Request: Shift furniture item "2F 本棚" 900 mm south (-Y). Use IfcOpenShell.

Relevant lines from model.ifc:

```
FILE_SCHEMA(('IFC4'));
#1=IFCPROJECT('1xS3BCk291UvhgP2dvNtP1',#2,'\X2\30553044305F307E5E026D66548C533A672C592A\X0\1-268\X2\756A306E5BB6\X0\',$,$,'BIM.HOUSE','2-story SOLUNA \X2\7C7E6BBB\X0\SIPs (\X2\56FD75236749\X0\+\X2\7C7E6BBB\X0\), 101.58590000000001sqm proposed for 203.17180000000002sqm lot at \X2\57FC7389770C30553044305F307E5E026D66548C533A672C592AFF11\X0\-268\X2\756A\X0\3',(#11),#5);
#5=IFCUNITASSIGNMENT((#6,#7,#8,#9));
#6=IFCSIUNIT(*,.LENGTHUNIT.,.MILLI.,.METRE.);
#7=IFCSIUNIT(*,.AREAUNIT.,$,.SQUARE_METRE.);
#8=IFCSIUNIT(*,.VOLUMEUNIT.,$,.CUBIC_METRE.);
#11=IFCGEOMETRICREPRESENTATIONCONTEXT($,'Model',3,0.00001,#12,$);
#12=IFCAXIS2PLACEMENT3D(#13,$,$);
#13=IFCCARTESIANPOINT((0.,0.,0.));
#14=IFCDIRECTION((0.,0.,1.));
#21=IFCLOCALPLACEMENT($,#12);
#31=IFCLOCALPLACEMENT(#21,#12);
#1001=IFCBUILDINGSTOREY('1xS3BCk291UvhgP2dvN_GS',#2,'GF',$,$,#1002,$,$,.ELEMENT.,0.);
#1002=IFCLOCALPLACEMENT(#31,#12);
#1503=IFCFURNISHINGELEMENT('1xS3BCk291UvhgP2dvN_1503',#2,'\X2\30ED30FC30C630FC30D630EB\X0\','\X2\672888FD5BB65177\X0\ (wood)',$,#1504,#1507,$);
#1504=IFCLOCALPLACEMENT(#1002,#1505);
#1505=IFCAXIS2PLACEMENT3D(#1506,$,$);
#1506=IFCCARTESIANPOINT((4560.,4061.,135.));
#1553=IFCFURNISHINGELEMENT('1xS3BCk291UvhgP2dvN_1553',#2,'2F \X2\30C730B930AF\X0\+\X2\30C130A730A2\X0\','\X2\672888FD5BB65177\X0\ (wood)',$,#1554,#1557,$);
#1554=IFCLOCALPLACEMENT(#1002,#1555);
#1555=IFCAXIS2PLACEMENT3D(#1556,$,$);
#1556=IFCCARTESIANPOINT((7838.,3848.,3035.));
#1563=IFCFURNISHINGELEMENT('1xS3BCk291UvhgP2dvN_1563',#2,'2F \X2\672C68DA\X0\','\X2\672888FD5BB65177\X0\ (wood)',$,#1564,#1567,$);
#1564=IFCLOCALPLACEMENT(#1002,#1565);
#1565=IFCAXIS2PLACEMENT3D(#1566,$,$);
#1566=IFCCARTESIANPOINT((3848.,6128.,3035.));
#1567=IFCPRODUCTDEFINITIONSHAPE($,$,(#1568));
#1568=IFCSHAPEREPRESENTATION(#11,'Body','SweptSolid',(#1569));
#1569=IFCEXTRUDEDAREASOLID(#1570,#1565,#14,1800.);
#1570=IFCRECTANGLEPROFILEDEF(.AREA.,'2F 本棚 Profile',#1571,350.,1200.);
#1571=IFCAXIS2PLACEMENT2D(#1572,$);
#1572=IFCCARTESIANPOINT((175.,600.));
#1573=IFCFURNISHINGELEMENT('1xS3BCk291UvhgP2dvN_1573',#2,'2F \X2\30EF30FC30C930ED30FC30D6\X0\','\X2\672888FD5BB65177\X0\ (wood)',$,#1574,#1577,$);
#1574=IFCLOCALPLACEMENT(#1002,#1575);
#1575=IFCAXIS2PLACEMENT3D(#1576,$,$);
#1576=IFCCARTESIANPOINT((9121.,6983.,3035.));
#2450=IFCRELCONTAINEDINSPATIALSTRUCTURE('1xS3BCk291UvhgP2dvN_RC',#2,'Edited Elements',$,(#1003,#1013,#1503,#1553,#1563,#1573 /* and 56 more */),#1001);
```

```python
import ifcopenshell
import ifcopenshell.api.geometry
import ifcopenshell.util.placement

model = ifcopenshell.open("model.ifc")

item = model.by_guid("1xS3BCk291UvhgP2dvN_1563")
matrix = ifcopenshell.util.placement.get_local_placement(item.ObjectPlacement)
matrix[1, 3] -= 900.0
ifcopenshell.api.geometry.edit_object_placement(model, product=item, matrix=matrix, is_si=False)

print(ifcopenshell.util.placement.get_local_placement(item.ObjectPlacement).round(3) + 0.0)

model.write("model-out.ifc")
```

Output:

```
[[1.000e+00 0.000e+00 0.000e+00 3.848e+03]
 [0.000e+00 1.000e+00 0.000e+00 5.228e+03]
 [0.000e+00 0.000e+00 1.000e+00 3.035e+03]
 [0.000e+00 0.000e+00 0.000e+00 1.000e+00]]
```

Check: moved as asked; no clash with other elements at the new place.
